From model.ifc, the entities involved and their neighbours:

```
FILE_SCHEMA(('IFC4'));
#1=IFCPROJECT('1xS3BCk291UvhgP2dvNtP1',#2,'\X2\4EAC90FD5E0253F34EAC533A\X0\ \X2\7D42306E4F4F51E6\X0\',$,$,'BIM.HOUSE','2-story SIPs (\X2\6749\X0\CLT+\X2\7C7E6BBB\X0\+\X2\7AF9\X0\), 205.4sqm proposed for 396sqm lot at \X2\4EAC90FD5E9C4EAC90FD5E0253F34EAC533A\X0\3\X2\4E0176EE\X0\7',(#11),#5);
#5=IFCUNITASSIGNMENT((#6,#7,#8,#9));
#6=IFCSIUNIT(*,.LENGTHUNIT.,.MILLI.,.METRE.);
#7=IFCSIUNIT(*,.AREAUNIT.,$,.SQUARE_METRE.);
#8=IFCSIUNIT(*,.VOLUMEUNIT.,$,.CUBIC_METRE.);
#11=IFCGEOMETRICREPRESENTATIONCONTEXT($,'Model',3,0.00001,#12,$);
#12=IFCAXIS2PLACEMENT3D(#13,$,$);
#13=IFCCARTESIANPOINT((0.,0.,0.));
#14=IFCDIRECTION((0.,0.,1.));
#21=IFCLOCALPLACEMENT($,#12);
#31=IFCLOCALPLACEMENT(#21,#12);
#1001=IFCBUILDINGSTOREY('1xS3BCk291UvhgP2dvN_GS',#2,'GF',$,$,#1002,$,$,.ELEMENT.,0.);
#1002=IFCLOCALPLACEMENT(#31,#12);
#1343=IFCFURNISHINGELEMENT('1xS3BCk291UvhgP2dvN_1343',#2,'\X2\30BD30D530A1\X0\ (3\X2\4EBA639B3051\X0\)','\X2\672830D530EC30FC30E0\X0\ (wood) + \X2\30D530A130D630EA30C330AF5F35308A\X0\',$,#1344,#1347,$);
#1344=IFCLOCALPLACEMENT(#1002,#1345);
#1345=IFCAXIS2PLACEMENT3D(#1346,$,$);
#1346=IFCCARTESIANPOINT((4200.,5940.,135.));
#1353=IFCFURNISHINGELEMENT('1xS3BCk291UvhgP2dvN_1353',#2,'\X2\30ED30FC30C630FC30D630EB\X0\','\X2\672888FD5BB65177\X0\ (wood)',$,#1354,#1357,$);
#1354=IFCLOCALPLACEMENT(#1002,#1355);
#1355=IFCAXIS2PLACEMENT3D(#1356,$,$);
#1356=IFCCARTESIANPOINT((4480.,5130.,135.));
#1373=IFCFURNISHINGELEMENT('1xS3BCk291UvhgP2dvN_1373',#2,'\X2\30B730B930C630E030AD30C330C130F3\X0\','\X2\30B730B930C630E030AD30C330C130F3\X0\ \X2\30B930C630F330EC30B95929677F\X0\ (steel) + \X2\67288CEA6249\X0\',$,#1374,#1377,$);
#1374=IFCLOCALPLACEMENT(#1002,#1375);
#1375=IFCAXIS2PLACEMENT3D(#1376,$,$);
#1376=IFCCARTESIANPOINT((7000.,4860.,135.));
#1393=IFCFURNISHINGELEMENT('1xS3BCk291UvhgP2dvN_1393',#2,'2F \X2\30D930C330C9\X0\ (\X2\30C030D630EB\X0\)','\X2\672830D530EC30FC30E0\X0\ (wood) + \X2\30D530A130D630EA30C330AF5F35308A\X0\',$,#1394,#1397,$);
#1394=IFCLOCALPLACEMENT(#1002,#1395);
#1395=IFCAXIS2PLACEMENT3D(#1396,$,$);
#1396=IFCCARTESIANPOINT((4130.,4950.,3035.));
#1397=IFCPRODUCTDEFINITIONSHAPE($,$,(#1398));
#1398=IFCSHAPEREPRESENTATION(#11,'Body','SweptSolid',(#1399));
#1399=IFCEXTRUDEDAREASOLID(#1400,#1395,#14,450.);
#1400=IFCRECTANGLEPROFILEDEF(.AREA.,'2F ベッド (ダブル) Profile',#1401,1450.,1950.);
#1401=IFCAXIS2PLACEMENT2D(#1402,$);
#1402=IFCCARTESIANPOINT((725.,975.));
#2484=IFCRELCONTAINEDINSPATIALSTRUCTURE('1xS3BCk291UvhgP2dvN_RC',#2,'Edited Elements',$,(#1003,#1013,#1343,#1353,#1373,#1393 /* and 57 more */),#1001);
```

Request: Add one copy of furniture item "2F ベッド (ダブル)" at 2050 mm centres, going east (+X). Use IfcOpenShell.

```python
import numpy as np
import ifcopenshell
import ifcopenshell.api.geometry
import ifcopenshell.api.root
import ifcopenshell.util.element
import ifcopenshell.util.placement

model = ifcopenshell.open("model.ifc")


def reuse_history(source, copy):
    """copy_class also copies each property set's owner history, people and application; keep the originals."""
    for rel in copy.IsDefinedBy:
        if rel.is_a("IfcRelDefinesByProperties") and (history := rel.RelatingPropertyDefinition.OwnerHistory):
            rel.RelatingPropertyDefinition.OwnerHistory = source.OwnerHistory
            ifcopenshell.util.element.remove_deep2(model, history)


source = model.by_guid("1xS3BCk291UvhgP2dvN_1393")
base = ifcopenshell.util.placement.get_local_placement(source.ObjectPlacement)
step = np.array([1.0, 0.0, 0.0]) * 2050.0

for i in range(1, 2):
    copy = ifcopenshell.api.root.copy_class(model, product=source)
    copy.Representation = ifcopenshell.util.element.copy_deep(
        model, source.Representation, exclude=["IfcGeometricRepresentationContext", "IfcRepresentationMap"]
    )
    reuse_history(source, copy)
    matrix = base.copy()
    matrix[:3, 3] += i * step
    print("added at", matrix[:3, 3].round(3) + 0.0)
    ifcopenshell.api.geometry.edit_object_placement(model, product=copy, matrix=matrix, is_si=False)

model.write("model_edited.ifc")
```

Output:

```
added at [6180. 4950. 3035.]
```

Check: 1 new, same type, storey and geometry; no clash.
